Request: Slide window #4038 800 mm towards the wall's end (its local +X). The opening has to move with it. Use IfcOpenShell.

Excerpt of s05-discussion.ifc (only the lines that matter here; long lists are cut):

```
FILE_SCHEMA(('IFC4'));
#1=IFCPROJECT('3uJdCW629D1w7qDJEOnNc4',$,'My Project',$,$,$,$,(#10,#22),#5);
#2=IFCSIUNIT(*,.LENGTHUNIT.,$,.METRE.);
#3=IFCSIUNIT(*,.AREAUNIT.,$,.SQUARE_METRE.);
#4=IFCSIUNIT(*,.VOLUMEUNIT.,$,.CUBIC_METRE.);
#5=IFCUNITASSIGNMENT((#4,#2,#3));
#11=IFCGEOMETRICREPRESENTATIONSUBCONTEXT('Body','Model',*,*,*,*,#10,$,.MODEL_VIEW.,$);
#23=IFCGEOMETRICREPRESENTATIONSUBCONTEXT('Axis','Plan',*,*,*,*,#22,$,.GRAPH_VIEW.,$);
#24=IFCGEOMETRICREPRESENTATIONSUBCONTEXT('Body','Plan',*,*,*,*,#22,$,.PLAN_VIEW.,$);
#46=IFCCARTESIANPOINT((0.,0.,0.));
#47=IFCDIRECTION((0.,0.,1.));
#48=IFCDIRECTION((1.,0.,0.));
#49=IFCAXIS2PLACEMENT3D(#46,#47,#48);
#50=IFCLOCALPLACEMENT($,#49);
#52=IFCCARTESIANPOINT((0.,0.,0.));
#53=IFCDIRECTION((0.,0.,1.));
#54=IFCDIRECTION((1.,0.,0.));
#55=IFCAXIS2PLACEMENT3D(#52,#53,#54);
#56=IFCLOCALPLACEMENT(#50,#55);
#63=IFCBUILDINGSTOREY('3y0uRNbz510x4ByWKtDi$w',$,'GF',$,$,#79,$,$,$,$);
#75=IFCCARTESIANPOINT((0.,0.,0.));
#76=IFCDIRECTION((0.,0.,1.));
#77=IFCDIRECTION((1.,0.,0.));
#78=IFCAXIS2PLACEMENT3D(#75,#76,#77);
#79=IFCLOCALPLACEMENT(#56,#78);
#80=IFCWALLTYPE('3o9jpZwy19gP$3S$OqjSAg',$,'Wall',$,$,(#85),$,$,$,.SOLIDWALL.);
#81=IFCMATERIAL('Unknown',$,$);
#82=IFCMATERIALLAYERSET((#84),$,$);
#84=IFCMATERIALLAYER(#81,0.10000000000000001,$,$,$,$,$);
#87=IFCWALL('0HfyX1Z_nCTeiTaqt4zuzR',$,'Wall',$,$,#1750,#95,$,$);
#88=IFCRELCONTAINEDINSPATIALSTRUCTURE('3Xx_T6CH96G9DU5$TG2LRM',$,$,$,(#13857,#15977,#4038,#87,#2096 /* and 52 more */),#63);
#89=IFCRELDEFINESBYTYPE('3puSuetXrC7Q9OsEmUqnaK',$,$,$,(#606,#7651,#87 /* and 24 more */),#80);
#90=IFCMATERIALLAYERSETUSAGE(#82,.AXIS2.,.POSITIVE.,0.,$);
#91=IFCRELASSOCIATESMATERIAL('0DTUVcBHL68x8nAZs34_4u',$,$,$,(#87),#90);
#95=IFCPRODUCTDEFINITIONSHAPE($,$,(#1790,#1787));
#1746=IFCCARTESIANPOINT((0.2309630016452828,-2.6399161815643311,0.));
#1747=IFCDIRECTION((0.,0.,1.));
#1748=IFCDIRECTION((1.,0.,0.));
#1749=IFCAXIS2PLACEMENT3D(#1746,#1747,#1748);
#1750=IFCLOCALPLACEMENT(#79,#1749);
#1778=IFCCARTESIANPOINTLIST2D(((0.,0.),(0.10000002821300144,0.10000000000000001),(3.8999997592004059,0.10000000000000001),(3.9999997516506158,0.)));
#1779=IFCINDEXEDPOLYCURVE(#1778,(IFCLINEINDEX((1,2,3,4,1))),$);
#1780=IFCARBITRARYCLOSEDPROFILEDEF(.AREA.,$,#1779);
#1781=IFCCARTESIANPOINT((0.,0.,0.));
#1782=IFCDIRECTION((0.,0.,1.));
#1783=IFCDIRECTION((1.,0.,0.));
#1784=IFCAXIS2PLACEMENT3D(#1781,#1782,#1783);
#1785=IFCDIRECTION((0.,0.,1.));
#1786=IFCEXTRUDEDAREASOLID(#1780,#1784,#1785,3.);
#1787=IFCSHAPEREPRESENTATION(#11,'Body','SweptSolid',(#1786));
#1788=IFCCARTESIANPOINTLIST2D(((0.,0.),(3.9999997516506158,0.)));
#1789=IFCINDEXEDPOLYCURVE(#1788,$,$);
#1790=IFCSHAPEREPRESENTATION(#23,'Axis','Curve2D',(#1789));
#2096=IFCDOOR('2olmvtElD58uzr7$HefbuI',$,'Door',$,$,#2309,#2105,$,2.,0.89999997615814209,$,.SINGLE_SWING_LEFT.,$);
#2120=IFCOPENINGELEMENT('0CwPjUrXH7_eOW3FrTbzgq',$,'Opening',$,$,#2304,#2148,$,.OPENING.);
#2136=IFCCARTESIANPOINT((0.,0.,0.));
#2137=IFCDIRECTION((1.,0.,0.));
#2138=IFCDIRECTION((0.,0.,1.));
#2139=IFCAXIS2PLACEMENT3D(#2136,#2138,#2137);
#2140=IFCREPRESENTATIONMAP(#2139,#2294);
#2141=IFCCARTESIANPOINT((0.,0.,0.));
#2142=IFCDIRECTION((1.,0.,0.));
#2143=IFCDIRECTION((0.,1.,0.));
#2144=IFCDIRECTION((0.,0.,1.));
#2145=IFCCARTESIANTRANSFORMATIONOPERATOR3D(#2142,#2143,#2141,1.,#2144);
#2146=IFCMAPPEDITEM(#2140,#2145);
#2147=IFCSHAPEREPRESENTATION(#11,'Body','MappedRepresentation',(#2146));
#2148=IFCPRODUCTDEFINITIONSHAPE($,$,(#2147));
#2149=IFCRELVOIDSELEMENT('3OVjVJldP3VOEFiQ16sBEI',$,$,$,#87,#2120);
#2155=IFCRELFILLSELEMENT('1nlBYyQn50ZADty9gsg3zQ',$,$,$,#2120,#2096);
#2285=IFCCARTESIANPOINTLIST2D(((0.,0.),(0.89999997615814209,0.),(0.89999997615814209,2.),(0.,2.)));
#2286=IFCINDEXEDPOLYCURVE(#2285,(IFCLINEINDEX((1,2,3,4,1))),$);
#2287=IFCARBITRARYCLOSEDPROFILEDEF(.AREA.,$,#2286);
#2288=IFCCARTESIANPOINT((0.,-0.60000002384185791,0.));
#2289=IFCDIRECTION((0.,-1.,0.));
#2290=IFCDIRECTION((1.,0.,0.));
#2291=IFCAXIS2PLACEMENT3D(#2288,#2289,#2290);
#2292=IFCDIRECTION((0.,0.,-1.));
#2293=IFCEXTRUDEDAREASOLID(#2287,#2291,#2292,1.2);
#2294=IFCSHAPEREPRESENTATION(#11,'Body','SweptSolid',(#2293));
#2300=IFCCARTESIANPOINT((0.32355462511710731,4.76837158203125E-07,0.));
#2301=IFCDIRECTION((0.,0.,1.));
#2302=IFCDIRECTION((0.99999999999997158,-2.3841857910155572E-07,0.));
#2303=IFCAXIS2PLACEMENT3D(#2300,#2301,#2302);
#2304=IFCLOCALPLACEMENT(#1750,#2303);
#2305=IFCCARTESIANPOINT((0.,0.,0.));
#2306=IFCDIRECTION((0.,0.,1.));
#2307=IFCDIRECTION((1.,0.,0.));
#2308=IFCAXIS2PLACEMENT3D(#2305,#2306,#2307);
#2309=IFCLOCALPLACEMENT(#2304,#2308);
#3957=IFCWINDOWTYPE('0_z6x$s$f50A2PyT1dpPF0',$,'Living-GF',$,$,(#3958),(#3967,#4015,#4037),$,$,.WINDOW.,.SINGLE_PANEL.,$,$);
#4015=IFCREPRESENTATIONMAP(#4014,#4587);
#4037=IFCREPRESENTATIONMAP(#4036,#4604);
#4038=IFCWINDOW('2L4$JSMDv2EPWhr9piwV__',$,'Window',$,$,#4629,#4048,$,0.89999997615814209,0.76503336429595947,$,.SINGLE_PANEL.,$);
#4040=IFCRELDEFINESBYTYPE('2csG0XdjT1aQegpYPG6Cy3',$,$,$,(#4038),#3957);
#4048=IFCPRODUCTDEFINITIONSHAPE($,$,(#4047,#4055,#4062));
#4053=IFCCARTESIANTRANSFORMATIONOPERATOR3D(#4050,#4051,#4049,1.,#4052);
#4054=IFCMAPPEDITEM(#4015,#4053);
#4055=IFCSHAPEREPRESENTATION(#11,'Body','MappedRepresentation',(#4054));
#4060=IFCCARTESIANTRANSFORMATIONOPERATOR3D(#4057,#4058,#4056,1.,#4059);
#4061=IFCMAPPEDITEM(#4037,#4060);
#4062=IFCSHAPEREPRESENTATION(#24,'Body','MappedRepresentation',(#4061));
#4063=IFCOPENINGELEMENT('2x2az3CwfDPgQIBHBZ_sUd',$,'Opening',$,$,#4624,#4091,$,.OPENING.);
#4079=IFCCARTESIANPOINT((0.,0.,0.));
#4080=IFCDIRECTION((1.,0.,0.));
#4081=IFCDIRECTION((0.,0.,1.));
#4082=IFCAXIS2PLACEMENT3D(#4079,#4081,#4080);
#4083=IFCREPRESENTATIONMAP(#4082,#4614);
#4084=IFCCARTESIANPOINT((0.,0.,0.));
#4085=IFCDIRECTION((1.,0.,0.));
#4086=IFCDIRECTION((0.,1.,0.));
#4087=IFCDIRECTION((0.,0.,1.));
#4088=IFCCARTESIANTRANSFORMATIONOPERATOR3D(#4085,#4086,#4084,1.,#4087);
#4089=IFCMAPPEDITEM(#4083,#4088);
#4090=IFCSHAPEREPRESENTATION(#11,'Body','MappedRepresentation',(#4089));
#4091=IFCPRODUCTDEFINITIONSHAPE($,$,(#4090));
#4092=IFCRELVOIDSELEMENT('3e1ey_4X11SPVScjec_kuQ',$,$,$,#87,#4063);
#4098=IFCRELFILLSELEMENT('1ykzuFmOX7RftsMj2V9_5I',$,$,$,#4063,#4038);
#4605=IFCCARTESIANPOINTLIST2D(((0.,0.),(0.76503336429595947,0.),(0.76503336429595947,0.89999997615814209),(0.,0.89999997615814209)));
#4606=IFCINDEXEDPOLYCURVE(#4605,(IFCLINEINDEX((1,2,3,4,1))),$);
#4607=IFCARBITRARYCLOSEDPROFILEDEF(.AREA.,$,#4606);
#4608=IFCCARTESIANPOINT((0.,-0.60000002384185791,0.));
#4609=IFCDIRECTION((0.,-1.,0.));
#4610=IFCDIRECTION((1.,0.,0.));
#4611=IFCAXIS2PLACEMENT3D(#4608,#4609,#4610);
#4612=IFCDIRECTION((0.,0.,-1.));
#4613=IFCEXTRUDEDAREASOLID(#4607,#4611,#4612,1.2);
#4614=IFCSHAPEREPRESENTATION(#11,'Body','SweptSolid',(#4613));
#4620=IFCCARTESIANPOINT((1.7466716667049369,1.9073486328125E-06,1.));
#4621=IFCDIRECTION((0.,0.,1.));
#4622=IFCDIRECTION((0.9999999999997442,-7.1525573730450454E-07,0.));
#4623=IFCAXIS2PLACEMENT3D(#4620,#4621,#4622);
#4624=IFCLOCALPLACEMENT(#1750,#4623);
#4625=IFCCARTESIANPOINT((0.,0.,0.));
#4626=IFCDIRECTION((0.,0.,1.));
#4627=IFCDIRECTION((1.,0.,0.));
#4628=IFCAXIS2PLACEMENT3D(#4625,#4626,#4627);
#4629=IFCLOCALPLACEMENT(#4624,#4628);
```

```python
import ifcopenshell
import ifcopenshell.api.geometry
import ifcopenshell.util.placement

model = ifcopenshell.open("s05-discussion.ifc")

window = model.by_guid("2L4$JSMDv2EPWhr9piwV__")
opening = window.FillsVoids[0].RelatingOpeningElement
wall = opening.VoidsElements[0].RelatingBuildingElement

wall_matrix = ifcopenshell.util.placement.get_local_placement(wall.ObjectPlacement)
shift = wall_matrix[:3, 0] * 0.8
before = ifcopenshell.util.placement.get_local_placement(window.ObjectPlacement)[:3, 3].copy()

# The window is placed relative to its opening, so it follows when the opening moves.
matrix = ifcopenshell.util.placement.get_local_placement(opening.ObjectPlacement)
matrix[:3, 3] += shift
ifcopenshell.api.geometry.edit_object_placement(
    model, product=opening, matrix=matrix, is_si=False, should_transform_children=True
)

after = ifcopenshell.util.placement.get_local_placement(window.ObjectPlacement)[:3, 3]
print("window moved by", (after - before).round(3) + 0.0)

model.write("s05-discussion_edited.ifc")
```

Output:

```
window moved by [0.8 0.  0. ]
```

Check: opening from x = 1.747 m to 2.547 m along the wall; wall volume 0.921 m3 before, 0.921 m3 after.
